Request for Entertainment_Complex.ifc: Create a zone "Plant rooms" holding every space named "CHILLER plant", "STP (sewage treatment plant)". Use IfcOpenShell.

First a look at what the model holds.

```python
import ifcopenshell

model = ifcopenshell.open("Entertainment_Complex.ifc")
print(model.schema)
seen = {}
for space in model.by_type("IfcSpace"):
    seen[space.LongName] = seen.get(space.LongName, 0) + 1
for name, count in sorted(seen.items(), key=str):
    print(count, "x", name)
print("zones:", [z.Name for z in model.by_type("IfcZone")][:20])
```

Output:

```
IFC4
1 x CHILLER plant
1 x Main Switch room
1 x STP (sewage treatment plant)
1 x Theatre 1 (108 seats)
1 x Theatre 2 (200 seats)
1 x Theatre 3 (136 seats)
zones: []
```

```python
import ifcopenshell
import ifcopenshell.api.group
import ifcopenshell.api.root

model = ifcopenshell.open("Entertainment_Complex.ifc")

names = {"CHILLER plant", "STP (sewage treatment plant)"}
spaces = [s for s in model.by_type("IfcSpace") if s.LongName in names]

zone = ifcopenshell.api.root.create_entity(model, ifc_class="IfcZone", name="Plant rooms")
ifcopenshell.api.group.assign_group(model, products=spaces, group=zone)
print(len(spaces), "spaces in", zone.Name)

model.write("Entertainment_Complex_edited.ifc")
```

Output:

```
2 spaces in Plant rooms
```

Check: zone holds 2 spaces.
